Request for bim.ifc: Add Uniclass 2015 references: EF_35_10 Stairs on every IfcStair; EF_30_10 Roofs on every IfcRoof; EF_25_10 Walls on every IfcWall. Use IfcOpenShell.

First a look at what the model holds.

```python
import ifcopenshell

model = ifcopenshell.open("bim.ifc")
print(model.schema)
print("classifications:", [c.Name for c in model.by_type("IfcClassification")])
for ifc_class in ("IfcDoor", "IfcRoof", "IfcStair", "IfcWall", "IfcWindow"):
    print(ifc_class, len(model.by_type(ifc_class)))
```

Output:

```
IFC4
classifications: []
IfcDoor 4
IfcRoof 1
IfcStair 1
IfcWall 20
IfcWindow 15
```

```python
import ifcopenshell
import ifcopenshell.api.classification

model = ifcopenshell.open("bim.ifc")

system = ifcopenshell.api.classification.add_classification(model, classification="Uniclass 2015")

codes = {
    "IfcStair": ("EF_35_10", "Stairs"),
    "IfcRoof": ("EF_30_10", "Roofs"),
    "IfcWall": ("EF_25_10", "Walls"),
}
for ifc_class, (code, name) in codes.items():
    products = model.by_type(ifc_class)
    ifcopenshell.api.classification.add_reference(
        model, products=products, classification=system, identification=code, name=name
    )
    print(code, len(products))

model.write("bim_updated.ifc")
```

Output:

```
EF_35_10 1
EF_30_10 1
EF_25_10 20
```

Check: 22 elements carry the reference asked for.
